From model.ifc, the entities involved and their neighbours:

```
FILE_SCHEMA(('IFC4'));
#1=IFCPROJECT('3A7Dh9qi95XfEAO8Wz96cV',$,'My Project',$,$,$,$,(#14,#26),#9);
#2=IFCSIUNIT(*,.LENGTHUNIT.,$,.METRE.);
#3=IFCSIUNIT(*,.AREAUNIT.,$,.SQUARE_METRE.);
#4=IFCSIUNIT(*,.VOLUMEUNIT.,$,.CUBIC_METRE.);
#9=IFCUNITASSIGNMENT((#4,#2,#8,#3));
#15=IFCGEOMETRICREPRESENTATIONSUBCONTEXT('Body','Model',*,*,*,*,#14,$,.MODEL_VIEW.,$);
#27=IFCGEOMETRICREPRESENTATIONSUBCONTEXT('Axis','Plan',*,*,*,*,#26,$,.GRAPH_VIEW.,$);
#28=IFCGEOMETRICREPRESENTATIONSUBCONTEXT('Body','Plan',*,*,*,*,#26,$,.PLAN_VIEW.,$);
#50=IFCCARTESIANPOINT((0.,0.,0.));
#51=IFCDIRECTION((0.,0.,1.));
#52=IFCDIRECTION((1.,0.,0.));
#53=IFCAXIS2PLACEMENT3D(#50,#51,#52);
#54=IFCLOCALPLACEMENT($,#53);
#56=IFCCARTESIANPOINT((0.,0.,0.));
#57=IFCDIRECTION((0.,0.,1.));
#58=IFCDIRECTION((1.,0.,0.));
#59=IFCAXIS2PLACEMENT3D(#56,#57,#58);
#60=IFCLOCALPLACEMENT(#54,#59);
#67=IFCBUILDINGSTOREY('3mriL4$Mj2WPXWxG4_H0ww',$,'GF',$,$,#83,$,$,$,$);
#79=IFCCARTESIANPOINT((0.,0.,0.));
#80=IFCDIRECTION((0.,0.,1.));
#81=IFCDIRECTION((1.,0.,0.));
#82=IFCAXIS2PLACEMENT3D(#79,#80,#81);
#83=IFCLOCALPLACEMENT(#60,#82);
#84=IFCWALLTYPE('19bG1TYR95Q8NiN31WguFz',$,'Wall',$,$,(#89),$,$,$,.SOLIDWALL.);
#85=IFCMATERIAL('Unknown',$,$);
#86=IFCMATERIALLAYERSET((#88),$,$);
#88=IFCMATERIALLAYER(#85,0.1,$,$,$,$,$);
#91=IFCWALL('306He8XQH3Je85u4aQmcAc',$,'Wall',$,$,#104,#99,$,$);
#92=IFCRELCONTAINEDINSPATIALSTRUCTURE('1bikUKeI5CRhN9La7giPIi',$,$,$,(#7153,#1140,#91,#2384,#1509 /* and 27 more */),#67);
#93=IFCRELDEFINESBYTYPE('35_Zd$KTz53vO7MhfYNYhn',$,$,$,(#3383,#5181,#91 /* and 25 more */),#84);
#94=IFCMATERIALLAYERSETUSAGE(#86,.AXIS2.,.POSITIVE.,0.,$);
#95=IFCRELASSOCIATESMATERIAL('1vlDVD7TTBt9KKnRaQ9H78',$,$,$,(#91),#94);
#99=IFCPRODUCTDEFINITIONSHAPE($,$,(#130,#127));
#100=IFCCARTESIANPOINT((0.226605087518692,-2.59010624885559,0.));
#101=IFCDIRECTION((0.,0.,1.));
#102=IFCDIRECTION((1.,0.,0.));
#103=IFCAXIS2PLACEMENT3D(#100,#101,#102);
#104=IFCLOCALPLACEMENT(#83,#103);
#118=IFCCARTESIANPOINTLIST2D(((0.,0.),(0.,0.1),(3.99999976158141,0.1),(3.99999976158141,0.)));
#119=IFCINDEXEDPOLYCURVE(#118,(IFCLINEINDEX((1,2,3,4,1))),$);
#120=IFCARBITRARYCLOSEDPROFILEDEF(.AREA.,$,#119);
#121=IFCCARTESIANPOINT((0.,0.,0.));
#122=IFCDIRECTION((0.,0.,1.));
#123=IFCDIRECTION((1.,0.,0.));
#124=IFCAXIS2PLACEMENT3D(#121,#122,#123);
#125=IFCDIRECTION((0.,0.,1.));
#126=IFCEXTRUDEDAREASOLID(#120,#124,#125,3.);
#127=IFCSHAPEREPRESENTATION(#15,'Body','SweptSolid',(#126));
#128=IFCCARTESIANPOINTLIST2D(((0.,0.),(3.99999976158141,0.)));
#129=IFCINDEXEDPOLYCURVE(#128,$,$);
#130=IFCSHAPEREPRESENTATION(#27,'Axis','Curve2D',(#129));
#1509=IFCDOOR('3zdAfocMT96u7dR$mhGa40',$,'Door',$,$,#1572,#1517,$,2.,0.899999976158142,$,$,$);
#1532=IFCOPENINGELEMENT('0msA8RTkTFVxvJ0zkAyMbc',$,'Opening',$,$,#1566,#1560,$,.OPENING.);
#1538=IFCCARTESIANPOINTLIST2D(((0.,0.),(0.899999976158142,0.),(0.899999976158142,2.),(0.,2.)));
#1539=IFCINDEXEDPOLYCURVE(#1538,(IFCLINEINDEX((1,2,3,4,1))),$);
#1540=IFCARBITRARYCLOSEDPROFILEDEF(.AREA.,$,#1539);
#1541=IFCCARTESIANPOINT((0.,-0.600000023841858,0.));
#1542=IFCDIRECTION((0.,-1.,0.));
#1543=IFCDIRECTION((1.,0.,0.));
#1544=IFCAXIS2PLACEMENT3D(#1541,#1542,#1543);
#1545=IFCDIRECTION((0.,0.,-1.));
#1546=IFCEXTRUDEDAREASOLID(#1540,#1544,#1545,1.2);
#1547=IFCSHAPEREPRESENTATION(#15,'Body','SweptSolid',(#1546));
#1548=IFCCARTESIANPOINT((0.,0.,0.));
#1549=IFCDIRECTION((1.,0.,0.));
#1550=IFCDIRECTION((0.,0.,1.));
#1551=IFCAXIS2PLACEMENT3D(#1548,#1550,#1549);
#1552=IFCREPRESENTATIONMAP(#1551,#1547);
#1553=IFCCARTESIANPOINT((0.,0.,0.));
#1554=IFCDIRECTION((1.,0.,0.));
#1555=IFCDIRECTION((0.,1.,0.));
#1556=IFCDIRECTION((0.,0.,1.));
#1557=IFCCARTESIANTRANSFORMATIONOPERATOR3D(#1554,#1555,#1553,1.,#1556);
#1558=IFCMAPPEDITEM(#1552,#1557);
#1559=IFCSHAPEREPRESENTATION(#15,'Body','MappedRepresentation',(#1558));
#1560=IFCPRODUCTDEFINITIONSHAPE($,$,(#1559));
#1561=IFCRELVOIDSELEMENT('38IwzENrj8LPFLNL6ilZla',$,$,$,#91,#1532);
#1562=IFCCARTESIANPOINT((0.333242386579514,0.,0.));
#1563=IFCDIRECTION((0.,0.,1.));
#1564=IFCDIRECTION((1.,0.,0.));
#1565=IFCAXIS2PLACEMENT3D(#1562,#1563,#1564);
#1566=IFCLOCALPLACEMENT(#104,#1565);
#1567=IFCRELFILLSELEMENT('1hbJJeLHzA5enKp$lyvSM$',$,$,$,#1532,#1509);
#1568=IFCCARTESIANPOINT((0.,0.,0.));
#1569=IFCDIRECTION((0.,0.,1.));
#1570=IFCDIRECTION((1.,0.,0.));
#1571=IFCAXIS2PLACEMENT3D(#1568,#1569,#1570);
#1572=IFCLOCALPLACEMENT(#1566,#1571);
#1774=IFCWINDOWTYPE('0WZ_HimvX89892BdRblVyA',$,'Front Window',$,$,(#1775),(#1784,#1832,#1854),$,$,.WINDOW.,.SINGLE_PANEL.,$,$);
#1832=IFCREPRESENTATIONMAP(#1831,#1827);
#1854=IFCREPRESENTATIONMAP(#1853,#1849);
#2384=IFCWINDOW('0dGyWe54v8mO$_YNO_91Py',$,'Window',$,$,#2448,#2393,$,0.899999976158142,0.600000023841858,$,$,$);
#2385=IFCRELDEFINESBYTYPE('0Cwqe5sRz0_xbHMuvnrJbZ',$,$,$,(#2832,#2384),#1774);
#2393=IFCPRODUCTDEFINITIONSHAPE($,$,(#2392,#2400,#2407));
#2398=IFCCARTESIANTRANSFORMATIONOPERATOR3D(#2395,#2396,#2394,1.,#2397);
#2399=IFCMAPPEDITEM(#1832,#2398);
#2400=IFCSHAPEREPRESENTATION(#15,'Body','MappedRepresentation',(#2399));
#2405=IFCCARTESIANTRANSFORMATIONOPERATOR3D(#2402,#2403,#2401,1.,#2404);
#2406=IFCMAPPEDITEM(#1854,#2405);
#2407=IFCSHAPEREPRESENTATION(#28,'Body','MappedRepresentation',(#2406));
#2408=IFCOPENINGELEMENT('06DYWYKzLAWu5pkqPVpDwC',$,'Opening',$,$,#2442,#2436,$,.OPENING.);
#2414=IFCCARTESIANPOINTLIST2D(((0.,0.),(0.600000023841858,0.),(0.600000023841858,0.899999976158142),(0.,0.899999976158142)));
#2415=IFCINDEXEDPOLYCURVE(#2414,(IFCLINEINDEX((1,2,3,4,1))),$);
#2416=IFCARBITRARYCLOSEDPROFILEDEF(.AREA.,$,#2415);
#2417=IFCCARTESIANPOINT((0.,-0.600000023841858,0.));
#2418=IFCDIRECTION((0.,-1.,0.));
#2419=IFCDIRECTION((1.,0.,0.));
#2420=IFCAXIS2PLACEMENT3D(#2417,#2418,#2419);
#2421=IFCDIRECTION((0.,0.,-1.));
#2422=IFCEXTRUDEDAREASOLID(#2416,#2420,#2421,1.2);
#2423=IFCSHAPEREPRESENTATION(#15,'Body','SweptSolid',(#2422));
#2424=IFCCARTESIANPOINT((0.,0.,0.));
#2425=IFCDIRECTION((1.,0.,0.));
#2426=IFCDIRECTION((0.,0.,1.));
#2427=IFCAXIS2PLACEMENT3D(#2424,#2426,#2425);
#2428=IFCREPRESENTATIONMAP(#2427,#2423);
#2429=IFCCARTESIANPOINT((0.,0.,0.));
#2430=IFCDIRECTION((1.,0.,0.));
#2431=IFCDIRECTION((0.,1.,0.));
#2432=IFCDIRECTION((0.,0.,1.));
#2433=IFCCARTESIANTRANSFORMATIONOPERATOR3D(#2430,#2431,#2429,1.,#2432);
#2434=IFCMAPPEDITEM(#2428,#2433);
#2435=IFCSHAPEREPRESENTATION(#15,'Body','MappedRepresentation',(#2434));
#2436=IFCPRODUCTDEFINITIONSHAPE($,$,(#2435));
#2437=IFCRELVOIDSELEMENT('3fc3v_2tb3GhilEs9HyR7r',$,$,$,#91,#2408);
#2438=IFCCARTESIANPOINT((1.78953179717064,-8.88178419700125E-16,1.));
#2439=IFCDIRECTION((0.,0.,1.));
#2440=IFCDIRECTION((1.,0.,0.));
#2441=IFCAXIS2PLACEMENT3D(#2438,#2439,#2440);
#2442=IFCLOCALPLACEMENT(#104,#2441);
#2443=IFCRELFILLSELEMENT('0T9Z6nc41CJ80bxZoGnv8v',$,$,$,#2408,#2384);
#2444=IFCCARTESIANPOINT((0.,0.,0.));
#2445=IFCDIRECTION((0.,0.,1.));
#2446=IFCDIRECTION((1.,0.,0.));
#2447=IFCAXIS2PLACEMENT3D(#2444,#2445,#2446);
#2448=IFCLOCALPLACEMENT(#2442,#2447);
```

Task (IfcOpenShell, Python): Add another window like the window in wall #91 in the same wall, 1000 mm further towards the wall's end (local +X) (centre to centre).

```python
import ifcopenshell
import ifcopenshell.api.feature
import ifcopenshell.api.geometry
import ifcopenshell.api.root
import ifcopenshell.geom
import ifcopenshell.util.element
import ifcopenshell.util.placement
import ifcopenshell.util.shape

model = ifcopenshell.open("model.ifc")
settings = ifcopenshell.geom.settings()


def volume(element):
    """Net volume in cubic metres, openings subtracted."""
    shape = ifcopenshell.geom.create_shape(settings, element)
    return ifcopenshell.util.shape.get_volume(shape.geometry)


window = model.by_id(2384)
opening = window.FillsVoids[0].RelatingOpeningElement
wall = opening.VoidsElements[0].RelatingBuildingElement
before = volume(wall)
shift = ifcopenshell.util.placement.get_local_placement(wall.ObjectPlacement)[:3, 0] * 1.0

# copy_class copies the void relationship, type, container and properties, but no geometry.
new_opening = ifcopenshell.api.root.copy_class(model, product=opening)
new_opening.Representation = ifcopenshell.util.element.copy_deep(
    model, opening.Representation, exclude=["IfcGeometricRepresentationContext", "IfcRepresentationMap"]
)
new_window = ifcopenshell.api.root.copy_class(model, product=window)
new_window.Representation = ifcopenshell.util.element.copy_deep(
    model, window.Representation, exclude=["IfcGeometricRepresentationContext", "IfcRepresentationMap"]
)
ifcopenshell.api.feature.add_filling(model, opening=new_opening, element=new_window)

for old, new in ((opening, new_opening), (window, new_window)):
    matrix = ifcopenshell.util.placement.get_local_placement(old.ObjectPlacement)
    matrix[:3, 3] += shift
    ifcopenshell.api.geometry.edit_object_placement(model, product=new, matrix=matrix, is_si=False)

after = volume(wall)

print(f"wall volume {before:.3f} -> {after:.3f} m3")

model.write("model_v2.ifc")
```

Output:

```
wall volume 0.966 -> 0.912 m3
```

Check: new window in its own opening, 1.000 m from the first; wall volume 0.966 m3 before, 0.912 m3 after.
